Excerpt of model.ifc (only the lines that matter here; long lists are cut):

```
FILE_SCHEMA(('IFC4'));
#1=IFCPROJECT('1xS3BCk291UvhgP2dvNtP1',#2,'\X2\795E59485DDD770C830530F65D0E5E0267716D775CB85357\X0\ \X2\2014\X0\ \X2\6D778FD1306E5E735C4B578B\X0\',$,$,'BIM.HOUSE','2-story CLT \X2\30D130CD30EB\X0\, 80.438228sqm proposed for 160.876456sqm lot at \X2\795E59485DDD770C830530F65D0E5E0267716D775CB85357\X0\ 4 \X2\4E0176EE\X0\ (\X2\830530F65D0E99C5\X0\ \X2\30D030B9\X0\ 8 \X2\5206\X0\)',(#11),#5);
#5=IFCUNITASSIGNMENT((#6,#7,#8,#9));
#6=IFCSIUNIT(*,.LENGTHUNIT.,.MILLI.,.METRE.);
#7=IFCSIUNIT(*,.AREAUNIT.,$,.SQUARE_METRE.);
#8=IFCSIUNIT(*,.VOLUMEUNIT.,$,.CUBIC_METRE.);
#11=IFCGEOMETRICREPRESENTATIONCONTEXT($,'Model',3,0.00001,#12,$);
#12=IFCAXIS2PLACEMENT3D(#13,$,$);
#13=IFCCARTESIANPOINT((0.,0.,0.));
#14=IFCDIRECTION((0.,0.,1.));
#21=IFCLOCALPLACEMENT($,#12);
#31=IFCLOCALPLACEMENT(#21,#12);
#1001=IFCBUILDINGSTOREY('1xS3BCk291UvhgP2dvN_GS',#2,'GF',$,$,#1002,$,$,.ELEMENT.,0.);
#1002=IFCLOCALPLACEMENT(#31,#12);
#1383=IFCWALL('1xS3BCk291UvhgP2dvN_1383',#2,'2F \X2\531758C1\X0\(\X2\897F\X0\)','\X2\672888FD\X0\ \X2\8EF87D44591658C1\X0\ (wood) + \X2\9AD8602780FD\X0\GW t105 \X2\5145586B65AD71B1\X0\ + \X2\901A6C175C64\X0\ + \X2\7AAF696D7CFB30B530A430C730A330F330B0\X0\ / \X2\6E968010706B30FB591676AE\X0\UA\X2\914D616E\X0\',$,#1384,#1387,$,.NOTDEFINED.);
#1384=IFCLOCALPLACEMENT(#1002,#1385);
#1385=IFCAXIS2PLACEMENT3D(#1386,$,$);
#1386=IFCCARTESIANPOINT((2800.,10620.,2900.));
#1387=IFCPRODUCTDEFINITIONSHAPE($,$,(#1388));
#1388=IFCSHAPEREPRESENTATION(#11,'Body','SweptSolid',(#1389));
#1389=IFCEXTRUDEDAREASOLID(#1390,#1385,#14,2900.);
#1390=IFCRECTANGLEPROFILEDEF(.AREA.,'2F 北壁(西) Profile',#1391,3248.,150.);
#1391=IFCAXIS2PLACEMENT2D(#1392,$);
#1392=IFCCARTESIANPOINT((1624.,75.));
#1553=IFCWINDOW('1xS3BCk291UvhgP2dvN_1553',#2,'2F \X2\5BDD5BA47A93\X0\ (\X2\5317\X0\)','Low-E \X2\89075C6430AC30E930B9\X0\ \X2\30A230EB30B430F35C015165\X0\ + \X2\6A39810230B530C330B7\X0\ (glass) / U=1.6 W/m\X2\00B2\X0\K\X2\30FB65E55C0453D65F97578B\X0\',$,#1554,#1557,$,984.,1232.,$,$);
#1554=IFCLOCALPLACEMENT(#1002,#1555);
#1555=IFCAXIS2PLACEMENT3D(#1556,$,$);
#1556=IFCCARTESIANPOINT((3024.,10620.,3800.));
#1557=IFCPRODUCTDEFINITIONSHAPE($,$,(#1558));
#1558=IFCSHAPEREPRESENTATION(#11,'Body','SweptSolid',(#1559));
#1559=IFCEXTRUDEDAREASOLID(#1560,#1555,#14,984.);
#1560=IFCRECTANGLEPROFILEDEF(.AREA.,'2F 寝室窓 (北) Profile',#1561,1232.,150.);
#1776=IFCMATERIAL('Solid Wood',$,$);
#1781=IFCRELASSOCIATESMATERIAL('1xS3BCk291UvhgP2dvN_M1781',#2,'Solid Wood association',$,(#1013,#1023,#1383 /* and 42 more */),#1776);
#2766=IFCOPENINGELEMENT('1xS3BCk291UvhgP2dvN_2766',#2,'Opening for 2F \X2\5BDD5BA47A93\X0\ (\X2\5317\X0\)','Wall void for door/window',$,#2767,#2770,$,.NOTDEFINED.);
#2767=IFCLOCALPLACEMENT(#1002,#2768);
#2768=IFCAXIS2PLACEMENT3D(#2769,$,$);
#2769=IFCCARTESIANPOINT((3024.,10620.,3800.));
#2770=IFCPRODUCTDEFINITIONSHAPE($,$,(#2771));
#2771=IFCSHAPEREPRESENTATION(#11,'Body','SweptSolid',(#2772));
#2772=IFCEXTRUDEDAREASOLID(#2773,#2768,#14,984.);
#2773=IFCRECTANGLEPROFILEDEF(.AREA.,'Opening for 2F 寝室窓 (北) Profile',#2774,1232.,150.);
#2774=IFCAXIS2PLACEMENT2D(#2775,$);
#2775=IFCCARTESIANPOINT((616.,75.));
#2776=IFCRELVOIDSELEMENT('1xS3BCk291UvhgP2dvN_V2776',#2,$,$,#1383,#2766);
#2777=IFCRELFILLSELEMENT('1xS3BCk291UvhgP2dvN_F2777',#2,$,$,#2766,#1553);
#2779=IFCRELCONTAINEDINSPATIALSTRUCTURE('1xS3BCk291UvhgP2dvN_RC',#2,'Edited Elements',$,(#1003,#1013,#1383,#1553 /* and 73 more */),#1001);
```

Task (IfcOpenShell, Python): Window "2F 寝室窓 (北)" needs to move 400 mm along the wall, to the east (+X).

```python
import ifcopenshell
import ifcopenshell.api.geometry
import ifcopenshell.util.placement

model = ifcopenshell.open("model.ifc")

window = model.by_guid("1xS3BCk291UvhgP2dvN_1553")
opening = window.FillsVoids[0].RelatingOpeningElement
wall = opening.VoidsElements[0].RelatingBuildingElement

wall_matrix = ifcopenshell.util.placement.get_local_placement(wall.ObjectPlacement)
shift = wall_matrix[:3, 0] * 400.0
before = ifcopenshell.util.placement.get_local_placement(window.ObjectPlacement)[:3, 3].copy()

# The window is not placed relative to its opening, so move both.
for product in (opening, window):
    matrix = ifcopenshell.util.placement.get_local_placement(product.ObjectPlacement)
    matrix[:3, 3] += shift
    ifcopenshell.api.geometry.edit_object_placement(model, product=product, matrix=matrix, is_si=False)

after = ifcopenshell.util.placement.get_local_placement(window.ObjectPlacement)[:3, 3]
print("window moved by", (after - before).round(3) + 0.0)

model.write("model_edited.ifc")
```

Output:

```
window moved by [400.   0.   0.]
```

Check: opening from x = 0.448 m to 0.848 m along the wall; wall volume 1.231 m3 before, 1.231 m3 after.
